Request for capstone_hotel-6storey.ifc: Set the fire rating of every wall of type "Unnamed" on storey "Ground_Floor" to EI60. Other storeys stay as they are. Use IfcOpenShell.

First a look at what the model holds.

```python
import ifcopenshell
import ifcopenshell.util.element

model = ifcopenshell.open("capstone_hotel-6storey.ifc")
print(model.schema)
storey = next(s for s in model.by_type("IfcBuildingStorey") if s.Name == "Ground_Floor")
walls = [e for e in ifcopenshell.util.element.get_decomposition(storey) if e.is_a("IfcWall")]
seen = {}
for e in walls:
    element_type = ifcopenshell.util.element.get_type(e)
    key = (element_type.Name if element_type != e and element_type else None, ifcopenshell.util.element.get_pset(e, "Pset_WallCommon", "FireRating"))
    seen[key] = seen.get(key, 0) + 1
for (name, value), count in sorted(seen.items(), key=str):
    print(count, "x", name, "|", value)
```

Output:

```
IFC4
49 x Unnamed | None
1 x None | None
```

```python
import ifcopenshell
import ifcopenshell.api.pset
import ifcopenshell.util.element

model = ifcopenshell.open("capstone_hotel-6storey.ifc")

storey = next(s for s in model.by_type("IfcBuildingStorey") if s.Name == "Ground_Floor")
walls = [e for e in ifcopenshell.util.element.get_decomposition(storey) if e.is_a("IfcWall")]

count = 0
for e in walls:
    element_type = ifcopenshell.util.element.get_type(e)
    if element_type in (None, e) or element_type.Name != "Unnamed":
        continue
    # add_pset returns the element's existing set when there is one.
    pset = ifcopenshell.api.pset.add_pset(model, product=e, name="Pset_WallCommon")
    ifcopenshell.api.pset.edit_pset(model, pset=pset, properties={"FireRating": "EI60"})
    count += 1

print(count, "walls updated")

model.write("capstone_hotel-6storey_v2.ifc")
```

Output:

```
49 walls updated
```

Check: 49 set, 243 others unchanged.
